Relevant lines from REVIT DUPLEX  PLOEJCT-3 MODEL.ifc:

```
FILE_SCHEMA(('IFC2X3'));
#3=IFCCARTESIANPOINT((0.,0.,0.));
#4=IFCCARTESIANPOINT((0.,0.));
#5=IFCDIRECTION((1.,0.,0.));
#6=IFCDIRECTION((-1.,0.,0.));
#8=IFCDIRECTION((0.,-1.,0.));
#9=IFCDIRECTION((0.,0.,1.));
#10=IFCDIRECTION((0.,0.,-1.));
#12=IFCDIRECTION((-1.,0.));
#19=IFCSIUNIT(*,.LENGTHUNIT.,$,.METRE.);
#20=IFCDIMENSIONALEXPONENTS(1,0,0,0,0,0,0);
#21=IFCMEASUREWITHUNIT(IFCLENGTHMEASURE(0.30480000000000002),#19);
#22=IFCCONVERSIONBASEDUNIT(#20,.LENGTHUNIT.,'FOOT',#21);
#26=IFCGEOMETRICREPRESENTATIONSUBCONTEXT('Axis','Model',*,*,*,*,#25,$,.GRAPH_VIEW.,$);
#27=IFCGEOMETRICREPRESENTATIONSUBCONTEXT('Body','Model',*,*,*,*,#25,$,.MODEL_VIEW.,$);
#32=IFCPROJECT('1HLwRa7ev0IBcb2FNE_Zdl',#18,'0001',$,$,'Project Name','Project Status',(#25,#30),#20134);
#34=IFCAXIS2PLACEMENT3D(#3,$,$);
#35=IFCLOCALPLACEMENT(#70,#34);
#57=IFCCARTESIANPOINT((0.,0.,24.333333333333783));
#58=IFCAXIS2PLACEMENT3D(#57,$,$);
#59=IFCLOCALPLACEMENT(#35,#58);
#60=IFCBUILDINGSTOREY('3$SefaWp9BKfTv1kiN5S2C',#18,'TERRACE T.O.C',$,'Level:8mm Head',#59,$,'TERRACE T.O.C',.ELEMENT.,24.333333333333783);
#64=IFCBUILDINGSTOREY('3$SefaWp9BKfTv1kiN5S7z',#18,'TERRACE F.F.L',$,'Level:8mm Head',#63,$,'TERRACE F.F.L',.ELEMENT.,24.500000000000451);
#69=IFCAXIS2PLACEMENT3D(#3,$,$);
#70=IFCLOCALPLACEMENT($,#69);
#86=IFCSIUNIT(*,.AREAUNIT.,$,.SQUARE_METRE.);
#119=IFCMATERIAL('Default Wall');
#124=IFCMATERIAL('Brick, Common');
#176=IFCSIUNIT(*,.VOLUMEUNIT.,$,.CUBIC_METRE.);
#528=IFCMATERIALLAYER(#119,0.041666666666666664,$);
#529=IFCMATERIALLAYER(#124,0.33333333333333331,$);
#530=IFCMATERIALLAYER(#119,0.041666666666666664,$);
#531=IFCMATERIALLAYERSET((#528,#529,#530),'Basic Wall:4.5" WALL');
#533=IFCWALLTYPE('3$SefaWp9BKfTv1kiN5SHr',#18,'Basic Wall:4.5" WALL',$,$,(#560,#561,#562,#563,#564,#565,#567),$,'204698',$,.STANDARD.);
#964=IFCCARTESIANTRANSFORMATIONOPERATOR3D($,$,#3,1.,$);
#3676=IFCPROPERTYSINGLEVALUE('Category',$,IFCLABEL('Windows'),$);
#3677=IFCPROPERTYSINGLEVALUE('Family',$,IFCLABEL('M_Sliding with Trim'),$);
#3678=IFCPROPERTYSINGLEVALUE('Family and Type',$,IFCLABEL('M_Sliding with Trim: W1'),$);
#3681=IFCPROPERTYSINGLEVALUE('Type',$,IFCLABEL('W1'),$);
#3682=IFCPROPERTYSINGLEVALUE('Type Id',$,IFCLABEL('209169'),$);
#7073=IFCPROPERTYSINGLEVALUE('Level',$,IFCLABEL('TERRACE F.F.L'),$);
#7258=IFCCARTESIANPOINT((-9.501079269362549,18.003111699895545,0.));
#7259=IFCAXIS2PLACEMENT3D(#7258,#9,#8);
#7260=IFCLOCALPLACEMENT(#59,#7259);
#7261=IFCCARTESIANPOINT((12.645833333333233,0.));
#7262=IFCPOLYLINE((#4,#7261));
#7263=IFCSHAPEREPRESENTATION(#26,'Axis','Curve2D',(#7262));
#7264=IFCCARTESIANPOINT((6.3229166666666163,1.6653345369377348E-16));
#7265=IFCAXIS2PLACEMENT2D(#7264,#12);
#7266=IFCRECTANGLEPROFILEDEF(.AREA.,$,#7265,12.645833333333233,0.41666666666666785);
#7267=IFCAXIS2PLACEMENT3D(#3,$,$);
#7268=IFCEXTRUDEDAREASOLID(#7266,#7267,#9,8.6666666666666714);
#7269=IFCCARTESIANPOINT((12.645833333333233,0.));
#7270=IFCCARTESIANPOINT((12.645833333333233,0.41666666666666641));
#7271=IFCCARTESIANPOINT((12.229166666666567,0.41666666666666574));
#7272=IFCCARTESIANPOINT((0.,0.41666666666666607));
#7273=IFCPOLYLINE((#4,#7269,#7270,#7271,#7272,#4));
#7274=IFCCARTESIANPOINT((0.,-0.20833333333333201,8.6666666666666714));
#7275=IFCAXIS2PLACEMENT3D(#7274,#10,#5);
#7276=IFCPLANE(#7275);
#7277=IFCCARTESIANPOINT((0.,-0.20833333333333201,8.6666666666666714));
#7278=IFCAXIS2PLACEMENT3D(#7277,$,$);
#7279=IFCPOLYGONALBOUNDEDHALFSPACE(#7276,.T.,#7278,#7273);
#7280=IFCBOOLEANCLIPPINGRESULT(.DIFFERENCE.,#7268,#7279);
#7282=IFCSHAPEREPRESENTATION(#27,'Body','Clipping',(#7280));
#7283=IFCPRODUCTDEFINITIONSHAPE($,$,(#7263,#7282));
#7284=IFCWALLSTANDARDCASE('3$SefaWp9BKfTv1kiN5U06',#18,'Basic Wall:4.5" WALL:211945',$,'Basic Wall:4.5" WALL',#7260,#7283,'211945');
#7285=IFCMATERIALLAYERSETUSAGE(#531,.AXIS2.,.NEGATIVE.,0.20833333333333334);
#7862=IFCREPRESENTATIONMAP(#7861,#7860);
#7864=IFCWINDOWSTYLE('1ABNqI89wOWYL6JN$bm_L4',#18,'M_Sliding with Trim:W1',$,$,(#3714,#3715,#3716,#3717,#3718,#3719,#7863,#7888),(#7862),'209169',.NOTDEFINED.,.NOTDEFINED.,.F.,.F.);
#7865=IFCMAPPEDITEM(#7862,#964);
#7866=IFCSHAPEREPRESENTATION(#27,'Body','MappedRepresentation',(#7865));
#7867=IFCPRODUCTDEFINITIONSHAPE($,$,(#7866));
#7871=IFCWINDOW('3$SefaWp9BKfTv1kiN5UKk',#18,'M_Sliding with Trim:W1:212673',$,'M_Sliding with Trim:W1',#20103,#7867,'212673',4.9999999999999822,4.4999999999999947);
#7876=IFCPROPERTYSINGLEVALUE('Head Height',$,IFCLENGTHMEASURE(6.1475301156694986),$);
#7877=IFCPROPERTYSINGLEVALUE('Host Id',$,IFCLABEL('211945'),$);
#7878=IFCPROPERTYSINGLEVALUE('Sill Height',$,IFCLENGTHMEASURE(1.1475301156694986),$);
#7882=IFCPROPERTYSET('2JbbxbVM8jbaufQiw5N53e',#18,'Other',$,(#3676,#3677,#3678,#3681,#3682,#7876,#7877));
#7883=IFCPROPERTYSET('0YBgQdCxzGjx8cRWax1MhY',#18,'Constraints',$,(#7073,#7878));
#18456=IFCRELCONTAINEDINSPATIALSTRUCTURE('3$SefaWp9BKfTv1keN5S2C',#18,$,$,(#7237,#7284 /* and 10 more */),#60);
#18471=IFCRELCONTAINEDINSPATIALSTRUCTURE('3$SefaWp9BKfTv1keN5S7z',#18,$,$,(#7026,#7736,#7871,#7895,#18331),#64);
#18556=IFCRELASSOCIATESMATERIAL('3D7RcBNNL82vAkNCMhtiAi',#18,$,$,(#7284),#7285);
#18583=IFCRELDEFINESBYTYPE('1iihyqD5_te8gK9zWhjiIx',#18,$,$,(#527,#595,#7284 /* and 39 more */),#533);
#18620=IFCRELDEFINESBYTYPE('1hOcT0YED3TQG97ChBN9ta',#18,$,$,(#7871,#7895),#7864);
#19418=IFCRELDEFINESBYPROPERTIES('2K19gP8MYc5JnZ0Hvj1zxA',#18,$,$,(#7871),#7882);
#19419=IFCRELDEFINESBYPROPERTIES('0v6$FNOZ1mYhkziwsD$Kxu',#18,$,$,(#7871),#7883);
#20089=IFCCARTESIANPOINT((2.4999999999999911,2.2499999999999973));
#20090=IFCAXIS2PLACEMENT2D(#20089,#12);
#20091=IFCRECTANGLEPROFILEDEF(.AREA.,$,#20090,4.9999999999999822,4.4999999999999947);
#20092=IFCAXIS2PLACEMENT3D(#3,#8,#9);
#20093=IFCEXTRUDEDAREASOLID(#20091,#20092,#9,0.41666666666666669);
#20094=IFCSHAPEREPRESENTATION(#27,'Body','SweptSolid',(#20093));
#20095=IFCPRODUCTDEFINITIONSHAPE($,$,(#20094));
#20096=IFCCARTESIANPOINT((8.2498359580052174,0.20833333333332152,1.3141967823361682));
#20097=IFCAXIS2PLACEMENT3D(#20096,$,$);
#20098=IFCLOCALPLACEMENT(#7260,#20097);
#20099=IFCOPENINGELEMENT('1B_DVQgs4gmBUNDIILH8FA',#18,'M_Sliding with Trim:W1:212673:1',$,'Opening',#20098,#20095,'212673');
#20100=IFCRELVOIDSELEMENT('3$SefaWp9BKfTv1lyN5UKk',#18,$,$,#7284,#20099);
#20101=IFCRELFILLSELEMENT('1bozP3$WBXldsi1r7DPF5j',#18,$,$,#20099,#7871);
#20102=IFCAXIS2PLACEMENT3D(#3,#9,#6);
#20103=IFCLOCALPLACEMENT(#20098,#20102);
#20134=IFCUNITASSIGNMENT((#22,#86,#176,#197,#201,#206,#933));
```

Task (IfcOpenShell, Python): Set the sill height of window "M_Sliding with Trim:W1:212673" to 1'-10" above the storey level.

```python
import numpy as np
import ifcopenshell
import ifcopenshell.api.geometry
import ifcopenshell.api.pset
import ifcopenshell.geom
import ifcopenshell.util.element
import ifcopenshell.util.placement
import ifcopenshell.util.shape
import ifcopenshell.util.unit

model = ifcopenshell.open("REVIT DUPLEX  PLOEJCT-3 MODEL.ifc")
unit_scale = ifcopenshell.util.unit.calculate_unit_scale(model)

window = model.by_id(7871)
opening = window.FillsVoids[0].RelatingOpeningElement
storey = ifcopenshell.util.element.get_container(window, ifc_class="IfcBuildingStorey")
level = ifcopenshell.util.placement.get_local_placement(storey.ObjectPlacement)[2, 3]

# The opening's origin need not be at the sill, so measure its lowest point.
shape = ifcopenshell.geom.create_shape(ifcopenshell.geom.settings(), opening)
bottom = ifcopenshell.util.shape.get_shape_bottom_elevation(shape, shape.geometry) / unit_scale
dz = level + 22 * 0.0254 / unit_scale - bottom

shift = np.array([0.0, 0.0, dz])
# The window is placed relative to its opening, so it follows when the opening moves.
matrix = ifcopenshell.util.placement.get_local_placement(opening.ObjectPlacement)
matrix[:3, 3] += shift
ifcopenshell.api.geometry.edit_object_placement(
    model, product=opening, matrix=matrix, is_si=False, should_transform_children=True
)

# Keep the stored heights in step.
pset = model.by_id(ifcopenshell.util.element.get_pset(window, "Other", should_inherit=False)["id"])
ifcopenshell.api.pset.edit_pset(model, pset=pset, properties={
    "Head Height": model.create_entity("IfcLengthMeasure", ifcopenshell.util.element.get_pset(window, "Other", "Head Height") + dz),
})
pset = model.by_id(ifcopenshell.util.element.get_pset(window, "Constraints", should_inherit=False)["id"])
ifcopenshell.api.pset.edit_pset(model, pset=pset, properties={
    "Sill Height": model.create_entity("IfcLengthMeasure", ifcopenshell.util.element.get_pset(window, "Constraints", "Sill Height") + dz),
})

print(f"moved by {dz * unit_scale:+.3f} m")

model.write("REVIT DUPLEX  PLOEJCT-3 MODEL_edited.ifc")
```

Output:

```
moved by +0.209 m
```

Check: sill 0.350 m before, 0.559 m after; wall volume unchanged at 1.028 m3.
